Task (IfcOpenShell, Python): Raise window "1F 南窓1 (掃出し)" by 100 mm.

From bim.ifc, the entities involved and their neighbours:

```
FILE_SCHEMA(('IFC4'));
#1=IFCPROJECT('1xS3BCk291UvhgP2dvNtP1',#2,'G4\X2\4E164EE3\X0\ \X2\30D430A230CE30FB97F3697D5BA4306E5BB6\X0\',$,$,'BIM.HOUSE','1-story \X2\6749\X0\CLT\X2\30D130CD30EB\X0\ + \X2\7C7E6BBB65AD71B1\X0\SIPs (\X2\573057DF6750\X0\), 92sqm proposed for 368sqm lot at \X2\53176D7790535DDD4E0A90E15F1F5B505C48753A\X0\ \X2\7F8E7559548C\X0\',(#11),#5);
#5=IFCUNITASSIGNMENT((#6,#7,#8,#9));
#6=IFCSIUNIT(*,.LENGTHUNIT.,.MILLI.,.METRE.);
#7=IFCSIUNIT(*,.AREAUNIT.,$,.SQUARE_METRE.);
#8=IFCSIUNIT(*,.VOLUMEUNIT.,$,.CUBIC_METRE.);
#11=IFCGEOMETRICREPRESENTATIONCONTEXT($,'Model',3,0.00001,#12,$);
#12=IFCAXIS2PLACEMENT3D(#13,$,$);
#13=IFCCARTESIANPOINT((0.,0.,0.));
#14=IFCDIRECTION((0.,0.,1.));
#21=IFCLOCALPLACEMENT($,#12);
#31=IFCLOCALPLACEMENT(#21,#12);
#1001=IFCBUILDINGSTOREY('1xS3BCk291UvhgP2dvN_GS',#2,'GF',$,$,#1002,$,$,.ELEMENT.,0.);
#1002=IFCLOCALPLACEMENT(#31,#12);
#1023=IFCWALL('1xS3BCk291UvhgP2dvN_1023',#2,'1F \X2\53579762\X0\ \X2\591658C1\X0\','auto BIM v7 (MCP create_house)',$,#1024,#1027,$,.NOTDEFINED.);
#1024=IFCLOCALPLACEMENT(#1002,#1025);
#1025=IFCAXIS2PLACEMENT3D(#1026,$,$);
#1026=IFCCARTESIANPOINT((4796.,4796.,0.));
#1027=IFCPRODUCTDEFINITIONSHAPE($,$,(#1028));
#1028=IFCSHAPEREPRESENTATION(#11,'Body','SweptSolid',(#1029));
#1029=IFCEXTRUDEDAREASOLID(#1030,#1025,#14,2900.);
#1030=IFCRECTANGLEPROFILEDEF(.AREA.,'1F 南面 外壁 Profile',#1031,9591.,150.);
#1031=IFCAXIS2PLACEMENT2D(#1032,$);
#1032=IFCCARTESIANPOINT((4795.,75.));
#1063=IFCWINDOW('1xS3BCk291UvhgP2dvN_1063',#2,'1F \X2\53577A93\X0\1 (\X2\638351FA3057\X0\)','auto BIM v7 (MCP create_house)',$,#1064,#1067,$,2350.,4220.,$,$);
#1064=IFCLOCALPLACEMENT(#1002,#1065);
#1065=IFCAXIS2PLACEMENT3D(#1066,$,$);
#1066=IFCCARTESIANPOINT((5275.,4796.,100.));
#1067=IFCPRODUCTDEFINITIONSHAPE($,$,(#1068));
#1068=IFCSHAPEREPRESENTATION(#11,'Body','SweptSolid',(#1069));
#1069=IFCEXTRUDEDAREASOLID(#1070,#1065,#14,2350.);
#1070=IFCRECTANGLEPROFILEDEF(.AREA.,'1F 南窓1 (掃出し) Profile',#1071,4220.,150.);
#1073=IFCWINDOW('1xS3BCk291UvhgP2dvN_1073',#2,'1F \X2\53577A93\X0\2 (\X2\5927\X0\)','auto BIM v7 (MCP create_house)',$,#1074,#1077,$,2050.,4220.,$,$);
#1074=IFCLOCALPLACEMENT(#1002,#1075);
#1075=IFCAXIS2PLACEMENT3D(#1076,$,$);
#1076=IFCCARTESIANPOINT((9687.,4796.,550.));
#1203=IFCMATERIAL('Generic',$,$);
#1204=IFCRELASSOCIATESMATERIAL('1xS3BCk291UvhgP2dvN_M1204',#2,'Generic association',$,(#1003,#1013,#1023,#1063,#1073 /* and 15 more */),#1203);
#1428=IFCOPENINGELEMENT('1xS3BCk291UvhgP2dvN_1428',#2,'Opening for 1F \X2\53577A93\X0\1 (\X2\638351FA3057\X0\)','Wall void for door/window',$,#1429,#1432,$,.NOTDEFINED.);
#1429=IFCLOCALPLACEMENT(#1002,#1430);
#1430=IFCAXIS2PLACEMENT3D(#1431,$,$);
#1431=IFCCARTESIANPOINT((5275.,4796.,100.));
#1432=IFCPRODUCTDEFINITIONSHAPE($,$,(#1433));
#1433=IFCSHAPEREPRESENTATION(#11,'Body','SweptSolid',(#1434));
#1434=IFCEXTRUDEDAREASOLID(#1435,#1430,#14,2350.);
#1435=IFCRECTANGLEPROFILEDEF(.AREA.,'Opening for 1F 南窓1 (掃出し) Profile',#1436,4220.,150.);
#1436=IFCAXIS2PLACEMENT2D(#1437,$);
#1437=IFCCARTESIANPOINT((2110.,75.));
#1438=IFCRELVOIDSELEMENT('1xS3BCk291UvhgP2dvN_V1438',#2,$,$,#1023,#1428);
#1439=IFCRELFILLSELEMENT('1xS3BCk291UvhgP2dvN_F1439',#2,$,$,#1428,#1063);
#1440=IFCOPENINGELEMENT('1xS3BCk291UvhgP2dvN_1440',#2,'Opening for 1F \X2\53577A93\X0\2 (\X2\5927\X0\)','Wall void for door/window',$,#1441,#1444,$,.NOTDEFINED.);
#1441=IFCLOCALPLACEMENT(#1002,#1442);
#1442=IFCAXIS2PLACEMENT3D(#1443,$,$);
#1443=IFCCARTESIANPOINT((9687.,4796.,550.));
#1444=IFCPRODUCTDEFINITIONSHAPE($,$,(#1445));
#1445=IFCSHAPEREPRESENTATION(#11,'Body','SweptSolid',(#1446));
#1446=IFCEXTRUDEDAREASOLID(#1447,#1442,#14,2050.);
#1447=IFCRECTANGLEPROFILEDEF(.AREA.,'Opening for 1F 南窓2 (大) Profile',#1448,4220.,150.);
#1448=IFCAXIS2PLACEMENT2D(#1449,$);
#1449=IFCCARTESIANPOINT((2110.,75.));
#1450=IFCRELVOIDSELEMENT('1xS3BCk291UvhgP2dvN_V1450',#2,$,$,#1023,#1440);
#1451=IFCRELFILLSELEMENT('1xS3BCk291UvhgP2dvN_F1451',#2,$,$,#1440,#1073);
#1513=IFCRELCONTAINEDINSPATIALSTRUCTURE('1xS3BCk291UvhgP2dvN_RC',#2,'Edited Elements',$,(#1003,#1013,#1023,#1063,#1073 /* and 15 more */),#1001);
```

```python
import numpy as np
import ifcopenshell
import ifcopenshell.api.geometry
import ifcopenshell.util.placement
import ifcopenshell.util.unit

model = ifcopenshell.open("bim.ifc")
unit_scale = ifcopenshell.util.unit.calculate_unit_scale(model)

window = model.by_guid("1xS3BCk291UvhgP2dvN_1063")
opening = window.FillsVoids[0].RelatingOpeningElement
dz = 0.1 / unit_scale

shift = np.array([0.0, 0.0, dz])
# The window is not placed relative to its opening, so move both.
for product in (opening, window):
    matrix = ifcopenshell.util.placement.get_local_placement(product.ObjectPlacement)
    matrix[:3, 3] += shift
    ifcopenshell.api.geometry.edit_object_placement(model, product=product, matrix=matrix, is_si=False)

print(f"moved by {dz * unit_scale:+.3f} m")

model.write("bim_rev.ifc")
```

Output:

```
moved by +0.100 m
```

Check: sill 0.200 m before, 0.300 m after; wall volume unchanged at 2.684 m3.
